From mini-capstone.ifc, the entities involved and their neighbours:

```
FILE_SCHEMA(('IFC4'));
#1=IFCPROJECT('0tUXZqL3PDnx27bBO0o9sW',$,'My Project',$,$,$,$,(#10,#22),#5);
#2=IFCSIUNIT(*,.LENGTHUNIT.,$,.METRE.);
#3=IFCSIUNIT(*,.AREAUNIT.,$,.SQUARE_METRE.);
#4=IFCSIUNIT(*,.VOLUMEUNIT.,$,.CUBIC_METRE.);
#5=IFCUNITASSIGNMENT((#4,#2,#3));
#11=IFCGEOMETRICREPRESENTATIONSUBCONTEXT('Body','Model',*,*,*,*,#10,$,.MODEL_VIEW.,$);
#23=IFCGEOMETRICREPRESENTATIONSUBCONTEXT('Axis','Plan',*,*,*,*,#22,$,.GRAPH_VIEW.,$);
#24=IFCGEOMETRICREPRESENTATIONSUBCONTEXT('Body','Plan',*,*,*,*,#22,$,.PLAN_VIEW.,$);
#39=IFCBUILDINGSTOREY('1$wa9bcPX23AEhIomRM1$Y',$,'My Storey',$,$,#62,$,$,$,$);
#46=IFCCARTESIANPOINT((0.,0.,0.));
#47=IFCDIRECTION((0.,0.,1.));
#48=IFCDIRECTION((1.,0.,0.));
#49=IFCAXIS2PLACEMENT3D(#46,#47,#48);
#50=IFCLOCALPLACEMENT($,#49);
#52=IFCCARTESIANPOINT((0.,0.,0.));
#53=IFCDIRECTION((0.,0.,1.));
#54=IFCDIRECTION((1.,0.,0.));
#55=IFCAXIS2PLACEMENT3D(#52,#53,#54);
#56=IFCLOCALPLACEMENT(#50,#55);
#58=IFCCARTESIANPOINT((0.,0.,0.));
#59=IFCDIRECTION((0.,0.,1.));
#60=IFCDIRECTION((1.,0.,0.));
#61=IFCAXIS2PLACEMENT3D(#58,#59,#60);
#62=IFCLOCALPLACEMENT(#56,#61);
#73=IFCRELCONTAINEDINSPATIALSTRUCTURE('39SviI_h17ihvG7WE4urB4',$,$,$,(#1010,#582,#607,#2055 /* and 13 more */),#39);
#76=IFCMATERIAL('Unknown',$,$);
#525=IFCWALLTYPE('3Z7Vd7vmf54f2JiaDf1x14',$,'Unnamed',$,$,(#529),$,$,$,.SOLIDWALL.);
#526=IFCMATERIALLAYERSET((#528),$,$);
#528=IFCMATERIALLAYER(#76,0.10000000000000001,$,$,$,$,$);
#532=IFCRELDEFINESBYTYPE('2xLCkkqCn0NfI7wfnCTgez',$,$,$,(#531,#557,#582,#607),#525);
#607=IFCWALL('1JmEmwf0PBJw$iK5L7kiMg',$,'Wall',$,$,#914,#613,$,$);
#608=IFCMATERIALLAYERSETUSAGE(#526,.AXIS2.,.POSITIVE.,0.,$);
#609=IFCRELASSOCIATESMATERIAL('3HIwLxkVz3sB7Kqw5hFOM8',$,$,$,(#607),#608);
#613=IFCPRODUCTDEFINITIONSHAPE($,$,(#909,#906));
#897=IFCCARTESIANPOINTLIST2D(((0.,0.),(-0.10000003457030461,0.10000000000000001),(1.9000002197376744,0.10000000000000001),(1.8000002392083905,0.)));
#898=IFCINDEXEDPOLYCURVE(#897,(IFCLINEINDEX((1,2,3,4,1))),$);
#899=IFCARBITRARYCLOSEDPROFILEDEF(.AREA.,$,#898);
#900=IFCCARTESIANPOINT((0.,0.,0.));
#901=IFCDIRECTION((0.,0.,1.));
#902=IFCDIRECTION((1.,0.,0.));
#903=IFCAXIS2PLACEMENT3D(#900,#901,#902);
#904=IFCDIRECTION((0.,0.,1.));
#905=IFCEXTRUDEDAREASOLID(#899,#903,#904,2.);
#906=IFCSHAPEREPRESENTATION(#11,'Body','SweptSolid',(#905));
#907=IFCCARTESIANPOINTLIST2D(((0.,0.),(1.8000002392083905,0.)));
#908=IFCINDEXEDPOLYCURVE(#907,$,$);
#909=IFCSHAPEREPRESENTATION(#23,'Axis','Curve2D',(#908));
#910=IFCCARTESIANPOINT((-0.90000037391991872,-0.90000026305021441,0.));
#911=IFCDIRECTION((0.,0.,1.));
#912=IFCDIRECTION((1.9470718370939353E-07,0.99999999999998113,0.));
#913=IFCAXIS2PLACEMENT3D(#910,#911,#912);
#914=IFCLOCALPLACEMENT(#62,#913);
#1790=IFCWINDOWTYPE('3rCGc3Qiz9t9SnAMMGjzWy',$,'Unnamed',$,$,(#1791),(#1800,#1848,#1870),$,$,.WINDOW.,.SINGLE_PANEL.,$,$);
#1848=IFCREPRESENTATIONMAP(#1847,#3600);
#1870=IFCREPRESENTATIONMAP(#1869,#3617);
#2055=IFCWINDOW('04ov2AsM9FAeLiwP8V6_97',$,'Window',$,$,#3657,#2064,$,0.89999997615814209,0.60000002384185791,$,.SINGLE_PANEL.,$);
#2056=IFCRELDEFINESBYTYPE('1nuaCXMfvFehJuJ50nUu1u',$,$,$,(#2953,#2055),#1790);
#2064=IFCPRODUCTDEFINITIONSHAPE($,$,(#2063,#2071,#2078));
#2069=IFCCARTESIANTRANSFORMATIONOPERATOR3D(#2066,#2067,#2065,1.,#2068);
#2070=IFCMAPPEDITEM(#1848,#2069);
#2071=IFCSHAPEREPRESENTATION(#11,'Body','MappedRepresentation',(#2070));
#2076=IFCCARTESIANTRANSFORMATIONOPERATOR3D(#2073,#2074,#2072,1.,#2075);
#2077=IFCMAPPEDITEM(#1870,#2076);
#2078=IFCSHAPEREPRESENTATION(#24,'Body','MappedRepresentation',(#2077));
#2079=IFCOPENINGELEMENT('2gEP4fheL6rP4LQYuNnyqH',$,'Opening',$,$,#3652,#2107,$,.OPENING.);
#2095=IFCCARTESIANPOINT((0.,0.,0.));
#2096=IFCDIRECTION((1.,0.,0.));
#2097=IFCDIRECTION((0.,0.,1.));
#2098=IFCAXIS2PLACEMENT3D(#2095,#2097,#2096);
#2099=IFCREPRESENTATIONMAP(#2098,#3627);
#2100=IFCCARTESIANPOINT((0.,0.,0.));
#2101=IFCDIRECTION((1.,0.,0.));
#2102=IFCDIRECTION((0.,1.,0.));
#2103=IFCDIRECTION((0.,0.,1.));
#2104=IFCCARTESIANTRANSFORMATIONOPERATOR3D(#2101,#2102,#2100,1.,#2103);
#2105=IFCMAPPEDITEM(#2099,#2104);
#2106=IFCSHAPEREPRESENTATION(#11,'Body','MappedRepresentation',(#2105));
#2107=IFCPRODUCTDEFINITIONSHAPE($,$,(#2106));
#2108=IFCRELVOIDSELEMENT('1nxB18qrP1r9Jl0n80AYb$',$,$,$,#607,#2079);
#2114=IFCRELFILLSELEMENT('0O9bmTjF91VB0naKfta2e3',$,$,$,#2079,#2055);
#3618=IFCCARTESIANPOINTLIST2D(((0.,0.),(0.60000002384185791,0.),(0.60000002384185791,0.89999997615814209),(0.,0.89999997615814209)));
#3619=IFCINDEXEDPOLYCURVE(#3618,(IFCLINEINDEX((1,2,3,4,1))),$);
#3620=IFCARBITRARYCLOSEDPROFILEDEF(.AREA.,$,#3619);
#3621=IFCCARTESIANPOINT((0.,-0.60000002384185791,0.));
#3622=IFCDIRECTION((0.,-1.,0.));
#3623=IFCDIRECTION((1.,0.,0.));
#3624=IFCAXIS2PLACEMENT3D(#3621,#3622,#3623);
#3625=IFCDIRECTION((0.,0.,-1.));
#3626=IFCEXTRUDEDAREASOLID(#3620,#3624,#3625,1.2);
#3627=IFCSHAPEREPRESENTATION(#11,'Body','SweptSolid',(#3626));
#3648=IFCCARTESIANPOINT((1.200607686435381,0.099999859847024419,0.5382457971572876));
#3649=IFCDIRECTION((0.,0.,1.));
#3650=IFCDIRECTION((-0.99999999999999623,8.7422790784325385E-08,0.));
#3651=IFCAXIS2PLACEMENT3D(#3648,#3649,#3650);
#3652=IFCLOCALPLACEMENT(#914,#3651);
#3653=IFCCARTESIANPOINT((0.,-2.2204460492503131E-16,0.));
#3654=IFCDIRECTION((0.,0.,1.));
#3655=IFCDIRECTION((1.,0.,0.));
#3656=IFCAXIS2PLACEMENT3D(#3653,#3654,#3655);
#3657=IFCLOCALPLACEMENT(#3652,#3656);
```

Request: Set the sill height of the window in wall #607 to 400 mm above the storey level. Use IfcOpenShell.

```python
import numpy as np
import ifcopenshell
import ifcopenshell.api.geometry
import ifcopenshell.geom
import ifcopenshell.util.element
import ifcopenshell.util.placement
import ifcopenshell.util.shape
import ifcopenshell.util.unit

model = ifcopenshell.open("mini-capstone.ifc")
unit_scale = ifcopenshell.util.unit.calculate_unit_scale(model)

window = model.by_id(2055)
opening = window.FillsVoids[0].RelatingOpeningElement
storey = ifcopenshell.util.element.get_container(window, ifc_class="IfcBuildingStorey")
level = ifcopenshell.util.placement.get_local_placement(storey.ObjectPlacement)[2, 3]

# The opening's origin need not be at the sill, so measure its lowest point.
shape = ifcopenshell.geom.create_shape(ifcopenshell.geom.settings(), opening)
bottom = ifcopenshell.util.shape.get_shape_bottom_elevation(shape, shape.geometry) / unit_scale
dz = level + 0.4 / unit_scale - bottom

shift = np.array([0.0, 0.0, dz])
# The window is placed relative to its opening, so it follows when the opening moves.
matrix = ifcopenshell.util.placement.get_local_placement(opening.ObjectPlacement)
matrix[:3, 3] += shift
ifcopenshell.api.geometry.edit_object_placement(
    model, product=opening, matrix=matrix, is_si=False, should_transform_children=True
)

print(f"moved by {dz * unit_scale:+.3f} m")

model.write("mini-capstone-out.ifc")
```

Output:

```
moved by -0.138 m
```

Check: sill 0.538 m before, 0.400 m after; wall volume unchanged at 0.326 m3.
